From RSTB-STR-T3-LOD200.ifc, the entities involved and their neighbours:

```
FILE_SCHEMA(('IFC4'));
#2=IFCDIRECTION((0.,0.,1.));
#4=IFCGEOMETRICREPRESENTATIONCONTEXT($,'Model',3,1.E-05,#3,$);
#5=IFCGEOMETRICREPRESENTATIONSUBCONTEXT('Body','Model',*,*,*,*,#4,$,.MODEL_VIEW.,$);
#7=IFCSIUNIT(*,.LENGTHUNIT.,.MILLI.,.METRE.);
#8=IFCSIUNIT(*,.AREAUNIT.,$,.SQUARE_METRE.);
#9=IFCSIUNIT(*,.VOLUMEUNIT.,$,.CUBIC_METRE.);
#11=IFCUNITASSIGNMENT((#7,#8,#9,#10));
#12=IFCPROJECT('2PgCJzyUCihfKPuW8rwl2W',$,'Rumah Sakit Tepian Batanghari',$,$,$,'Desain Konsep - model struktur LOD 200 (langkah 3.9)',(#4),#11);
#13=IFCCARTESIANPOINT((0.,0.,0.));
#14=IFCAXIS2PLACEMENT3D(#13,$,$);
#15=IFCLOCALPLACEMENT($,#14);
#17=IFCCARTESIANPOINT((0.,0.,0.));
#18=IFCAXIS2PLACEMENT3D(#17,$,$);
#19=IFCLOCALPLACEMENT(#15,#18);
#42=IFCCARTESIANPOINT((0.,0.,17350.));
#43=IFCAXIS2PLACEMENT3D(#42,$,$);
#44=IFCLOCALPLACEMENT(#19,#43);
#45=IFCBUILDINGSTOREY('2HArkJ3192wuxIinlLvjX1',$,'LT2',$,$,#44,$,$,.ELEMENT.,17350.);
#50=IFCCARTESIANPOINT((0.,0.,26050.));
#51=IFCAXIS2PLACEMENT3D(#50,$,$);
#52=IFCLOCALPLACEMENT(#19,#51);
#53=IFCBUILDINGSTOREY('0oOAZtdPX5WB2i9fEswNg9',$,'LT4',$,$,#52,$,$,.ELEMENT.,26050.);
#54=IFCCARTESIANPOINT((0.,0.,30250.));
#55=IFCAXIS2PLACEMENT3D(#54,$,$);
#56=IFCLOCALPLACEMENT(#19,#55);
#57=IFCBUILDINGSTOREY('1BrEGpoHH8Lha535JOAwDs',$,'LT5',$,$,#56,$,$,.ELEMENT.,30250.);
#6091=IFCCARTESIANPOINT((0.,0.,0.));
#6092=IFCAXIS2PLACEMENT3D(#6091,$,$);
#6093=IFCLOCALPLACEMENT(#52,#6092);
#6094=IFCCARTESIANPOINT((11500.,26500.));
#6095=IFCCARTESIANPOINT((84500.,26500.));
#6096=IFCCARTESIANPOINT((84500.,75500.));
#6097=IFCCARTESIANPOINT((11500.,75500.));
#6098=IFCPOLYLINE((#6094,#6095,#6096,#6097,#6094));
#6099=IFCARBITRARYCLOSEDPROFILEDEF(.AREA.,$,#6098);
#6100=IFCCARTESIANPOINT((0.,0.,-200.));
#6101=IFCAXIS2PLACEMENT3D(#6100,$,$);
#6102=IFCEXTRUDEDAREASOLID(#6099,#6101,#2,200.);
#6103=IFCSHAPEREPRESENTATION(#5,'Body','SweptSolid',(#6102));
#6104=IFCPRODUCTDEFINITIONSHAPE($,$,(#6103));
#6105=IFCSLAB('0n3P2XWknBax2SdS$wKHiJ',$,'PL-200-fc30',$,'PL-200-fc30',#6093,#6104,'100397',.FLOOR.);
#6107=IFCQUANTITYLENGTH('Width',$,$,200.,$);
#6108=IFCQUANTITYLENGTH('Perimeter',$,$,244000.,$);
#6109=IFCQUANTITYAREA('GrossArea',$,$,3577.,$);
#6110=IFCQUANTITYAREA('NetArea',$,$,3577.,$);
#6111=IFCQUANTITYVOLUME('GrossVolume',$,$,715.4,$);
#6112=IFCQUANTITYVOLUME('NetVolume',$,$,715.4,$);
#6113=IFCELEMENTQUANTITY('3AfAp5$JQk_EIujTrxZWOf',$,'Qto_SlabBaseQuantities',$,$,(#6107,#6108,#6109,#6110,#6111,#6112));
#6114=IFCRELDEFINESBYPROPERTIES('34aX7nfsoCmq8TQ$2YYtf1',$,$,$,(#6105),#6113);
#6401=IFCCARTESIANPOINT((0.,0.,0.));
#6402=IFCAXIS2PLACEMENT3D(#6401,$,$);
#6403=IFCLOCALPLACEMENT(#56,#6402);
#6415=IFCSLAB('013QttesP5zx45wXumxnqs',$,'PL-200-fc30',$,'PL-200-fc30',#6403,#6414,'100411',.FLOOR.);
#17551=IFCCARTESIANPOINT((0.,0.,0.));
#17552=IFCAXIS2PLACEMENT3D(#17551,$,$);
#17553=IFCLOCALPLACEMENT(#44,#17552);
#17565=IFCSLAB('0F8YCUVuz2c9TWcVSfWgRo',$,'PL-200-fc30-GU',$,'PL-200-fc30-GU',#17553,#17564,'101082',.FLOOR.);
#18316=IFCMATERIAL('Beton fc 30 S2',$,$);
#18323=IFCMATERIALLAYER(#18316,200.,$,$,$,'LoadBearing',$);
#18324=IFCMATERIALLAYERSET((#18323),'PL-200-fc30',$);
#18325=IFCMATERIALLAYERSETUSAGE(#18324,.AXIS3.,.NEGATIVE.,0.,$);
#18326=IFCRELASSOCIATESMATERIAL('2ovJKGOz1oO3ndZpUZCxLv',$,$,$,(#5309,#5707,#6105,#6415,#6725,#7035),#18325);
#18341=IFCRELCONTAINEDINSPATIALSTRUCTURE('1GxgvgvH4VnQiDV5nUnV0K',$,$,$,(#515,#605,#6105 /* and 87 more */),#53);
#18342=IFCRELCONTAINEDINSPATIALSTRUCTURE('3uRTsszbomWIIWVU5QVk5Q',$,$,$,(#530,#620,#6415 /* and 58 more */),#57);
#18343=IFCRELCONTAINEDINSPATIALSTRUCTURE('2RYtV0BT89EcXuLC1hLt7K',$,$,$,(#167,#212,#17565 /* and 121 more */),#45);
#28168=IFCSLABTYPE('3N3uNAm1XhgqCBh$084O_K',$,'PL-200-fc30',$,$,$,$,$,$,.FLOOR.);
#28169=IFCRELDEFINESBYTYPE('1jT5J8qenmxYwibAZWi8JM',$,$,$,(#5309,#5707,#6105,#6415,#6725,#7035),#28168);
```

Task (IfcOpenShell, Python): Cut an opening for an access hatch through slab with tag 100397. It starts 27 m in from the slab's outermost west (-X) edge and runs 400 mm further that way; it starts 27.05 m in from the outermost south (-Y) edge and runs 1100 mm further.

```python
import numpy as np
import ifcopenshell
import ifcopenshell.api.feature
import ifcopenshell.api.geometry
import ifcopenshell.api.pset
import ifcopenshell.api.root
import ifcopenshell.geom
import ifcopenshell.util.element
import ifcopenshell.util.placement
import ifcopenshell.util.representation
import ifcopenshell.util.shape
import ifcopenshell.util.unit

model = ifcopenshell.open("RSTB-STR-T3-LOD200.ifc")
unit_scale = ifcopenshell.util.unit.calculate_unit_scale(model)
area_scale = ifcopenshell.util.unit.calculate_unit_scale(model, "AREAUNIT")
volume_scale = ifcopenshell.util.unit.calculate_unit_scale(model, "VOLUMEUNIT")
settings = ifcopenshell.geom.settings()


def volume(element):
    """Net volume in cubic metres, openings subtracted."""
    shape = ifcopenshell.geom.create_shape(settings, element)
    return ifcopenshell.util.shape.get_volume(shape.geometry)


slab = model.by_guid("0n3P2XWknBax2SdS$wKHiJ")
before = volume(slab)

# Extent in the slab's own axes, in metres. The edges named are its -X and -Y sides.
slab_shape = ifcopenshell.geom.create_shape(settings, slab)
vertices = ifcopenshell.util.shape.get_vertices(slab_shape.geometry)
x_min, y_min, bottom = vertices.min(axis=0)
top = vertices[:, 2].max()

opening = ifcopenshell.api.root.create_entity(model, ifc_class="IfcOpeningElement", name="Access hatch opening", predefined_type="OPENING")
context = ifcopenshell.util.representation.get_context(model, "Model", "Body", "MODEL_VIEW")
width, depth = 0.4, 1.1
outline = [(0.0, 0.0), (width, 0.0), (width, depth), (0.0, depth), (0.0, 0.0)]
# Overshoot both faces by 50 mm so the cut is clean.
shape = ifcopenshell.api.geometry.add_slab_representation(
    model, context=context, depth=top - bottom + 0.1, polyline=outline
)
ifcopenshell.api.geometry.assign_representation(model, product=opening, representation=shape)

matrix = ifcopenshell.util.placement.get_local_placement(slab.ObjectPlacement)
matrix[:, 3] = matrix @ np.append(np.array([x_min + 27, y_min + 27.05, bottom - 0.05]) / unit_scale, 1.0)
ifcopenshell.api.geometry.edit_object_placement(model, product=opening, matrix=matrix, is_si=False)
ifcopenshell.api.feature.add_feature(model, feature=opening, element=slab)

after = volume(slab)

# Update the slab's stored quantities.
qto = model.by_id(ifcopenshell.util.element.get_pset(slab, "Qto_SlabBaseQuantities", should_inherit=False)["id"])
ifcopenshell.api.pset.edit_qto(model, qto=qto, properties={
    "NetArea": after / (top - bottom) / area_scale,
    "NetVolume": after / volume_scale,
})

print(f"slab volume {before:.3f} -> {after:.3f} m3")

model.write("RSTB-STR-T3-LOD200_v2.ifc")
```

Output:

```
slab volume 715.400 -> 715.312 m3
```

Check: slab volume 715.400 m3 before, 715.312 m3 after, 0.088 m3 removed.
